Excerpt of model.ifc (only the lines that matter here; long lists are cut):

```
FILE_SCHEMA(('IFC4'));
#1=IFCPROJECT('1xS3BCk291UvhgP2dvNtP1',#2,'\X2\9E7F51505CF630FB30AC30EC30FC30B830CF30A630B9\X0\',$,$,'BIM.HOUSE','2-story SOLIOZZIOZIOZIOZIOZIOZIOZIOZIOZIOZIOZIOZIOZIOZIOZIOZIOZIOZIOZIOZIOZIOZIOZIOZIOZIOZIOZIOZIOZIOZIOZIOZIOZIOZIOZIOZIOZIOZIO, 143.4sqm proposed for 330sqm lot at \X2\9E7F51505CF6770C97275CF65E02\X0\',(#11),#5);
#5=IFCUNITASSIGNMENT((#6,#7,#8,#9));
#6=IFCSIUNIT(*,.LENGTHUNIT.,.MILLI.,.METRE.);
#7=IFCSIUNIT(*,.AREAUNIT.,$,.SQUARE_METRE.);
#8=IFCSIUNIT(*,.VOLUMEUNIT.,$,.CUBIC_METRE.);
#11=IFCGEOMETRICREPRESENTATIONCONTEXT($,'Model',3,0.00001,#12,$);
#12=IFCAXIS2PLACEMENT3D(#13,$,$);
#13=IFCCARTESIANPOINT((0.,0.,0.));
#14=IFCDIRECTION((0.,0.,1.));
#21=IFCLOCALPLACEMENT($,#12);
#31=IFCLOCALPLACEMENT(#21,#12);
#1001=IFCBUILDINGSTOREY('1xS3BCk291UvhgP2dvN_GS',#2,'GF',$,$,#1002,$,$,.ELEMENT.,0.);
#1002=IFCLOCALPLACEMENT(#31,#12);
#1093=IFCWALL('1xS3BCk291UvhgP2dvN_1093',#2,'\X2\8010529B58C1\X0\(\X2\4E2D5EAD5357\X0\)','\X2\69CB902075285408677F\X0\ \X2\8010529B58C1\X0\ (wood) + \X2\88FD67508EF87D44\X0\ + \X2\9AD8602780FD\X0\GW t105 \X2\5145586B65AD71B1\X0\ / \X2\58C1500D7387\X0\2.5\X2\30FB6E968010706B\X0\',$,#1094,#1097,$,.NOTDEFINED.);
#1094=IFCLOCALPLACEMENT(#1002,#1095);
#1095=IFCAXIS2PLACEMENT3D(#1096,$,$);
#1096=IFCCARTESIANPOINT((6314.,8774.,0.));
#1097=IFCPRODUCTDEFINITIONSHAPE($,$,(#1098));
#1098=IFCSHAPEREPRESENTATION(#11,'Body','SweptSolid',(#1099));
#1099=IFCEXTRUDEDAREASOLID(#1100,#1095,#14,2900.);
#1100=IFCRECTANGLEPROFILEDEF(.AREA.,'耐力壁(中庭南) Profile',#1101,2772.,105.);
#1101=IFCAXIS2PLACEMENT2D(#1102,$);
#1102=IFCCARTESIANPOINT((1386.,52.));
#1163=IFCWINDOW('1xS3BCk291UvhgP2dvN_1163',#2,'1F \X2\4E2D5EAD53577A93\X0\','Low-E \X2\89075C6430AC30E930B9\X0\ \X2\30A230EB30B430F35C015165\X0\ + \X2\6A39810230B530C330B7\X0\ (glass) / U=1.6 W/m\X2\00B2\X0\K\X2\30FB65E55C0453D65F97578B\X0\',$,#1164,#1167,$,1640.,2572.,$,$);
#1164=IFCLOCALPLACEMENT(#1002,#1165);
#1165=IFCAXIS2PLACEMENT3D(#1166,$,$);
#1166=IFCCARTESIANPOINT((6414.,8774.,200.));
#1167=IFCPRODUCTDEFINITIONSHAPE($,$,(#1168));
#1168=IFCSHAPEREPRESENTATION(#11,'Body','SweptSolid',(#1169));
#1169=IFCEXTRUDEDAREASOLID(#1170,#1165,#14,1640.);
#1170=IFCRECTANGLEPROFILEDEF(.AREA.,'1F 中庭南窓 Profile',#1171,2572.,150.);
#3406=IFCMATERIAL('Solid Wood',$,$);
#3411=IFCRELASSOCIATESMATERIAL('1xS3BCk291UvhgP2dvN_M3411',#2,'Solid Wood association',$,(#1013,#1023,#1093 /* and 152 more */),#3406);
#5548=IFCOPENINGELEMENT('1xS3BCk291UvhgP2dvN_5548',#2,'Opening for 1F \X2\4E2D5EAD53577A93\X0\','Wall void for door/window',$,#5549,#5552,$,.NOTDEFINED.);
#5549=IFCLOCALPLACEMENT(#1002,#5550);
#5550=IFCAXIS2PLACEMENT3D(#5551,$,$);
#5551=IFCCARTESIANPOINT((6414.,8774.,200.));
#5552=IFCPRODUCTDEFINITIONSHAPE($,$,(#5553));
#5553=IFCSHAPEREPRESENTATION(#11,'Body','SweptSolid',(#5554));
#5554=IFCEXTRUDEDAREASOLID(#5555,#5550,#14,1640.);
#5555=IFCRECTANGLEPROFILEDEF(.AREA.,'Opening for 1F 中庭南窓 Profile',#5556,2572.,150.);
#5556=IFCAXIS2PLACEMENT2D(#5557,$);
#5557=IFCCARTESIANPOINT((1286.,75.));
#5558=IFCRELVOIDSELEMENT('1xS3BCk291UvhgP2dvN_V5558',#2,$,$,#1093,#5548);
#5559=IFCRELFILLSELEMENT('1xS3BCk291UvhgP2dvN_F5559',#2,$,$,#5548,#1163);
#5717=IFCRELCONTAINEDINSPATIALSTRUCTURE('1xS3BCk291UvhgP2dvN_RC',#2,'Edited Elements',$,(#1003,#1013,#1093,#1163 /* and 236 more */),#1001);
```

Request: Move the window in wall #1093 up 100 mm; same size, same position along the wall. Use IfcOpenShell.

```python
import numpy as np
import ifcopenshell
import ifcopenshell.api.geometry
import ifcopenshell.util.placement
import ifcopenshell.util.unit

model = ifcopenshell.open("model.ifc")
unit_scale = ifcopenshell.util.unit.calculate_unit_scale(model)

window = model.by_guid("1xS3BCk291UvhgP2dvN_1163")
opening = window.FillsVoids[0].RelatingOpeningElement
dz = 0.1 / unit_scale

shift = np.array([0.0, 0.0, dz])
# The window is not placed relative to its opening, so move both.
for product in (opening, window):
    matrix = ifcopenshell.util.placement.get_local_placement(product.ObjectPlacement)
    matrix[:3, 3] += shift
    ifcopenshell.api.geometry.edit_object_placement(model, product=product, matrix=matrix, is_si=False)

print(f"moved by {dz * unit_scale:+.3f} m")

model.write("model-out.ifc")
```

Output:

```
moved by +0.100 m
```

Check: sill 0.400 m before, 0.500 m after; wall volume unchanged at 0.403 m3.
